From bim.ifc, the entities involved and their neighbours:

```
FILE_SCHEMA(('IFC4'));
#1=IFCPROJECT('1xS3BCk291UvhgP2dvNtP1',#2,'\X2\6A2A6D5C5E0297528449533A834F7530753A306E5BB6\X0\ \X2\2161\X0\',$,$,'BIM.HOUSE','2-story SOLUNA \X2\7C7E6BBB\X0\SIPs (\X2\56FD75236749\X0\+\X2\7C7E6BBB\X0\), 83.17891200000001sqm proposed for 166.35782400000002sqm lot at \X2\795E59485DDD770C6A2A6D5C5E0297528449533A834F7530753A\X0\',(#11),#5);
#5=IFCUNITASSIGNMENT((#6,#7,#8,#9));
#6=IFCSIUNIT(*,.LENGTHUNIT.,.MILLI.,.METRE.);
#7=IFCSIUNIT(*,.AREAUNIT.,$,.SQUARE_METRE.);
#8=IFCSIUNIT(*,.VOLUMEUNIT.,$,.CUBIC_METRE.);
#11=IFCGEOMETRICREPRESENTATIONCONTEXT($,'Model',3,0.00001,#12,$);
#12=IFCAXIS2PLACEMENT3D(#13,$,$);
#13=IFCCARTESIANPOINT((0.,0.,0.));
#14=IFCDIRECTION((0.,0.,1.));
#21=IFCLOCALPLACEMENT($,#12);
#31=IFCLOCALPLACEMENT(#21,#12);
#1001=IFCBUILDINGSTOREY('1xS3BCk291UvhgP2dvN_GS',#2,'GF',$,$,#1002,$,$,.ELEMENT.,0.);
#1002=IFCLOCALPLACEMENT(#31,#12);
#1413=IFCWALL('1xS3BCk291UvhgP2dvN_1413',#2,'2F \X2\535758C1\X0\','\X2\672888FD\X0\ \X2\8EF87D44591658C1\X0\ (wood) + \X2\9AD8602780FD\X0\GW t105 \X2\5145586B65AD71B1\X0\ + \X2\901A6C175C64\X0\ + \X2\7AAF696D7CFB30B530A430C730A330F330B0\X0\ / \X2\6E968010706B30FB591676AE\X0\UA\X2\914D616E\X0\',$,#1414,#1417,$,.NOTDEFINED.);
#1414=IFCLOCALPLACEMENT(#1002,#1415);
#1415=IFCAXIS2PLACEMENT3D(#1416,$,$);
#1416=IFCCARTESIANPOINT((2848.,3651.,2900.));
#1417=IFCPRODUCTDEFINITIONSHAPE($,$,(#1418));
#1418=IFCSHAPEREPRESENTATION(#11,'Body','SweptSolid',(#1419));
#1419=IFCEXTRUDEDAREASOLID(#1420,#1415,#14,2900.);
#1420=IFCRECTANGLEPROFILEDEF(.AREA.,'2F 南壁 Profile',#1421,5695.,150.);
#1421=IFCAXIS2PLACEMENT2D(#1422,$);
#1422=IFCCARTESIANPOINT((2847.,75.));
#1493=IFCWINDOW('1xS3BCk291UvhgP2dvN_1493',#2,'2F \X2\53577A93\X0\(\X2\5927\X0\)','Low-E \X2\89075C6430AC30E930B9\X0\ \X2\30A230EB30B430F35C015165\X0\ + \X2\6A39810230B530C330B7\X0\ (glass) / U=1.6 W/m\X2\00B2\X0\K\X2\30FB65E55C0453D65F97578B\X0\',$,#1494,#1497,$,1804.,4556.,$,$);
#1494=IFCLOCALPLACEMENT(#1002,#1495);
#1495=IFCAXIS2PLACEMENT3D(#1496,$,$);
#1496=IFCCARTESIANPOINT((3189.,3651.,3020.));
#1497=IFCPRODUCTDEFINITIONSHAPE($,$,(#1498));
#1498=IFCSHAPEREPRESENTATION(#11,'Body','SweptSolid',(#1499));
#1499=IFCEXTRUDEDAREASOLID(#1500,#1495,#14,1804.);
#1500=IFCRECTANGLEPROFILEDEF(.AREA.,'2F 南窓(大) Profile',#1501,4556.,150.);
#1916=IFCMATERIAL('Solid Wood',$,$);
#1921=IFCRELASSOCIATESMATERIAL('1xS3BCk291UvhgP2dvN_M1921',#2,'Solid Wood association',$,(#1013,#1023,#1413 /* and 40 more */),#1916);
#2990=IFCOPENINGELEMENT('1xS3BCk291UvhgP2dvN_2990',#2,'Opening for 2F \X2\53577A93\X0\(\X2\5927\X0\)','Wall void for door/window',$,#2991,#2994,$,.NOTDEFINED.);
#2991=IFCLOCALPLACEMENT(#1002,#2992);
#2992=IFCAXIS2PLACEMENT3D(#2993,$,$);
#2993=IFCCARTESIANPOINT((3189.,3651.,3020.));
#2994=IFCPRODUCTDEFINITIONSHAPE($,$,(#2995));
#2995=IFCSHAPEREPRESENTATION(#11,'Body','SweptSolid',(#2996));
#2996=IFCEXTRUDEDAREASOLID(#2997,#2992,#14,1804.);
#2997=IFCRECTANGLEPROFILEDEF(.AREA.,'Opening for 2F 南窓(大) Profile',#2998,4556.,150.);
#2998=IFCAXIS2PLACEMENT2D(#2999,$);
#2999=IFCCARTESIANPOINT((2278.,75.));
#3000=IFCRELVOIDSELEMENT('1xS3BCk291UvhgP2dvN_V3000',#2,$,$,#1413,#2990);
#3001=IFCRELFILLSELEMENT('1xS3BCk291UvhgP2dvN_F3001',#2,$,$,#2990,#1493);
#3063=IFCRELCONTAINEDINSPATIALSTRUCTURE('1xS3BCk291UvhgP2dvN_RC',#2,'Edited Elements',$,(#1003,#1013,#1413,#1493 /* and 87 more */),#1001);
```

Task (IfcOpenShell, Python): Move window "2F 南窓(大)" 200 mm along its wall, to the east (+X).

```python
import ifcopenshell
import ifcopenshell.api.geometry
import ifcopenshell.util.placement
import ifcopenshell.util.unit

model = ifcopenshell.open("bim.ifc")
unit_scale = ifcopenshell.util.unit.calculate_unit_scale(model)

window = model.by_guid("1xS3BCk291UvhgP2dvN_1493")
opening = window.FillsVoids[0].RelatingOpeningElement
wall = opening.VoidsElements[0].RelatingBuildingElement

wall_matrix = ifcopenshell.util.placement.get_local_placement(wall.ObjectPlacement)
shift = wall_matrix[:3, 0] * 0.2 / unit_scale
before = ifcopenshell.util.placement.get_local_placement(window.ObjectPlacement)[:3, 3].copy()

# The window is not placed relative to its opening, so move both.
for product in (opening, window):
    matrix = ifcopenshell.util.placement.get_local_placement(product.ObjectPlacement)
    matrix[:3, 3] += shift
    ifcopenshell.api.geometry.edit_object_placement(model, product=product, matrix=matrix, is_si=False)

after = ifcopenshell.util.placement.get_local_placement(window.ObjectPlacement)[:3, 3]
print("window moved by", (after - before).round(3) + 0.0)

model.write("bim-out.ifc")
```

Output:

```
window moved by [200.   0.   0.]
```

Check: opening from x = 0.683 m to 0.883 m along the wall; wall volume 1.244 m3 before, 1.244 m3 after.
